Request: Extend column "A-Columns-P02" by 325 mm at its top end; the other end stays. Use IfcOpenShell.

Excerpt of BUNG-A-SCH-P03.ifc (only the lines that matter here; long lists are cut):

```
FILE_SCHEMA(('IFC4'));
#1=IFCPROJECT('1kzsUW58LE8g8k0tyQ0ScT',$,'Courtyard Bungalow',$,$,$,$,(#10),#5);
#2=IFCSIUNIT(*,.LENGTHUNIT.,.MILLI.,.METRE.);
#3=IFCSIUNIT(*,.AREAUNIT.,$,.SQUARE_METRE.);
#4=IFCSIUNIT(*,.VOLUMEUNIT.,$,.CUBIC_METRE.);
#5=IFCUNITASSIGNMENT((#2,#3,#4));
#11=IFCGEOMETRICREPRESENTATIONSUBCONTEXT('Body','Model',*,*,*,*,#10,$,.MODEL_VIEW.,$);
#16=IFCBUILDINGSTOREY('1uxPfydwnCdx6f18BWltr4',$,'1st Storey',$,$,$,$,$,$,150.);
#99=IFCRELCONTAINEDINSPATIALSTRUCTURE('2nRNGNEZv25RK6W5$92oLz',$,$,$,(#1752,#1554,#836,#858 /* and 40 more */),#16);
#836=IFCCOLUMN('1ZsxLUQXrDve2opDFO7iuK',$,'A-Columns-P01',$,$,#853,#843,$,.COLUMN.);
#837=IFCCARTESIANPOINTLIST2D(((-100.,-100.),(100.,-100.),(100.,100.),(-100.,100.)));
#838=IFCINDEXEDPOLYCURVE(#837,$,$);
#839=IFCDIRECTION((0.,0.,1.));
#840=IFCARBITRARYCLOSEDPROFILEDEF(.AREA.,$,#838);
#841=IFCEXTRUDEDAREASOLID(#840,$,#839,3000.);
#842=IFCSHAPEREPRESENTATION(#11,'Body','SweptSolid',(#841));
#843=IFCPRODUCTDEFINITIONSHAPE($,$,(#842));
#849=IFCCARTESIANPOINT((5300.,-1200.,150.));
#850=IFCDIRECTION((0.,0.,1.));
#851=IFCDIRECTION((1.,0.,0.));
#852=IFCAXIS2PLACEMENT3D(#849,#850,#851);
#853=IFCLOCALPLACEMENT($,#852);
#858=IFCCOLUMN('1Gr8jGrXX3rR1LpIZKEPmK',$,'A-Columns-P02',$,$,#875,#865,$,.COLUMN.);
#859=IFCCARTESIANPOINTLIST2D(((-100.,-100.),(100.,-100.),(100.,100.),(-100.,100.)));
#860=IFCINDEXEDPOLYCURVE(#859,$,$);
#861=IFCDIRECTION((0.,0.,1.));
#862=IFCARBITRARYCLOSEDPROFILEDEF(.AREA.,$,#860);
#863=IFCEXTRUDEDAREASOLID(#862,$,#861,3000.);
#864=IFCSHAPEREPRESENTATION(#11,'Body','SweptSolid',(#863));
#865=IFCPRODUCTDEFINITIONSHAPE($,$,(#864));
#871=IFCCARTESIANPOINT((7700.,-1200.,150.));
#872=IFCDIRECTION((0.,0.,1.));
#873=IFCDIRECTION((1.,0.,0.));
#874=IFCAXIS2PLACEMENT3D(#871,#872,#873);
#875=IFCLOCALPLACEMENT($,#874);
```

```python
import ifcopenshell
import ifcopenshell.util.representation

model = ifcopenshell.open("BUNG-A-SCH-P03.ifc")

member = model.by_id(858)
change = 325.0

# The extrusion runs towards the end named, so only its depth changes.
body = ifcopenshell.util.representation.get_representation(member, "Model", "Body")
solid = body.Items[0]
old_length = solid.Depth
solid.Depth += change

print(f"length {old_length:g} -> {solid.Depth:g}")

model.write("BUNG-A-SCH-P03_updated.ifc")
```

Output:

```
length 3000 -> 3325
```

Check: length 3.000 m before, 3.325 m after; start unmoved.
